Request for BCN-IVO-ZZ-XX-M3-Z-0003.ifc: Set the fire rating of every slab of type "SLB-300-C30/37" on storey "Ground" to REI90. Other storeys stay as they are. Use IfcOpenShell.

First a look at what the model holds.

```python
import ifcopenshell
import ifcopenshell.util.element

model = ifcopenshell.open("BCN-IVO-ZZ-XX-M3-Z-0003.ifc")
print(model.schema)
storey = next(s for s in model.by_type("IfcBuildingStorey") if s.Name == "Ground")
slabs = [e for e in ifcopenshell.util.element.get_decomposition(storey) if e.is_a("IfcSlab")]
seen = {}
for e in slabs:
    element_type = ifcopenshell.util.element.get_type(e)
    key = (element_type.Name if element_type != e and element_type else None, ifcopenshell.util.element.get_pset(e, "Pset_SlabCommon", "FireRating"))
    seen[key] = seen.get(key, 0) + 1
for (name, value), count in sorted(seen.items(), key=str):
    print(count, "x", name, "|", value)
```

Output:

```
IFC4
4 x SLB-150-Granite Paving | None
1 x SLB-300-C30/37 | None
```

```python
import ifcopenshell
import ifcopenshell.api.pset
import ifcopenshell.util.element

model = ifcopenshell.open("BCN-IVO-ZZ-XX-M3-Z-0003.ifc")

storey = next(s for s in model.by_type("IfcBuildingStorey") if s.Name == "Ground")
slabs = [e for e in ifcopenshell.util.element.get_decomposition(storey) if e.is_a("IfcSlab")]

count = 0
for e in slabs:
    element_type = ifcopenshell.util.element.get_type(e)
    if element_type in (None, e) or element_type.Name != "SLB-300-C30/37":
        continue
    # add_pset returns the element's existing set when there is one.
    pset = ifcopenshell.api.pset.add_pset(model, product=e, name="Pset_SlabCommon")
    ifcopenshell.api.pset.edit_pset(model, pset=pset, properties={"FireRating": "REI90"})
    count += 1

print(count, "slabs updated")

model.write("BCN-IVO-ZZ-XX-M3-Z-0003-out.ifc")
```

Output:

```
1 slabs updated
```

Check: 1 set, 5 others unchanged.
